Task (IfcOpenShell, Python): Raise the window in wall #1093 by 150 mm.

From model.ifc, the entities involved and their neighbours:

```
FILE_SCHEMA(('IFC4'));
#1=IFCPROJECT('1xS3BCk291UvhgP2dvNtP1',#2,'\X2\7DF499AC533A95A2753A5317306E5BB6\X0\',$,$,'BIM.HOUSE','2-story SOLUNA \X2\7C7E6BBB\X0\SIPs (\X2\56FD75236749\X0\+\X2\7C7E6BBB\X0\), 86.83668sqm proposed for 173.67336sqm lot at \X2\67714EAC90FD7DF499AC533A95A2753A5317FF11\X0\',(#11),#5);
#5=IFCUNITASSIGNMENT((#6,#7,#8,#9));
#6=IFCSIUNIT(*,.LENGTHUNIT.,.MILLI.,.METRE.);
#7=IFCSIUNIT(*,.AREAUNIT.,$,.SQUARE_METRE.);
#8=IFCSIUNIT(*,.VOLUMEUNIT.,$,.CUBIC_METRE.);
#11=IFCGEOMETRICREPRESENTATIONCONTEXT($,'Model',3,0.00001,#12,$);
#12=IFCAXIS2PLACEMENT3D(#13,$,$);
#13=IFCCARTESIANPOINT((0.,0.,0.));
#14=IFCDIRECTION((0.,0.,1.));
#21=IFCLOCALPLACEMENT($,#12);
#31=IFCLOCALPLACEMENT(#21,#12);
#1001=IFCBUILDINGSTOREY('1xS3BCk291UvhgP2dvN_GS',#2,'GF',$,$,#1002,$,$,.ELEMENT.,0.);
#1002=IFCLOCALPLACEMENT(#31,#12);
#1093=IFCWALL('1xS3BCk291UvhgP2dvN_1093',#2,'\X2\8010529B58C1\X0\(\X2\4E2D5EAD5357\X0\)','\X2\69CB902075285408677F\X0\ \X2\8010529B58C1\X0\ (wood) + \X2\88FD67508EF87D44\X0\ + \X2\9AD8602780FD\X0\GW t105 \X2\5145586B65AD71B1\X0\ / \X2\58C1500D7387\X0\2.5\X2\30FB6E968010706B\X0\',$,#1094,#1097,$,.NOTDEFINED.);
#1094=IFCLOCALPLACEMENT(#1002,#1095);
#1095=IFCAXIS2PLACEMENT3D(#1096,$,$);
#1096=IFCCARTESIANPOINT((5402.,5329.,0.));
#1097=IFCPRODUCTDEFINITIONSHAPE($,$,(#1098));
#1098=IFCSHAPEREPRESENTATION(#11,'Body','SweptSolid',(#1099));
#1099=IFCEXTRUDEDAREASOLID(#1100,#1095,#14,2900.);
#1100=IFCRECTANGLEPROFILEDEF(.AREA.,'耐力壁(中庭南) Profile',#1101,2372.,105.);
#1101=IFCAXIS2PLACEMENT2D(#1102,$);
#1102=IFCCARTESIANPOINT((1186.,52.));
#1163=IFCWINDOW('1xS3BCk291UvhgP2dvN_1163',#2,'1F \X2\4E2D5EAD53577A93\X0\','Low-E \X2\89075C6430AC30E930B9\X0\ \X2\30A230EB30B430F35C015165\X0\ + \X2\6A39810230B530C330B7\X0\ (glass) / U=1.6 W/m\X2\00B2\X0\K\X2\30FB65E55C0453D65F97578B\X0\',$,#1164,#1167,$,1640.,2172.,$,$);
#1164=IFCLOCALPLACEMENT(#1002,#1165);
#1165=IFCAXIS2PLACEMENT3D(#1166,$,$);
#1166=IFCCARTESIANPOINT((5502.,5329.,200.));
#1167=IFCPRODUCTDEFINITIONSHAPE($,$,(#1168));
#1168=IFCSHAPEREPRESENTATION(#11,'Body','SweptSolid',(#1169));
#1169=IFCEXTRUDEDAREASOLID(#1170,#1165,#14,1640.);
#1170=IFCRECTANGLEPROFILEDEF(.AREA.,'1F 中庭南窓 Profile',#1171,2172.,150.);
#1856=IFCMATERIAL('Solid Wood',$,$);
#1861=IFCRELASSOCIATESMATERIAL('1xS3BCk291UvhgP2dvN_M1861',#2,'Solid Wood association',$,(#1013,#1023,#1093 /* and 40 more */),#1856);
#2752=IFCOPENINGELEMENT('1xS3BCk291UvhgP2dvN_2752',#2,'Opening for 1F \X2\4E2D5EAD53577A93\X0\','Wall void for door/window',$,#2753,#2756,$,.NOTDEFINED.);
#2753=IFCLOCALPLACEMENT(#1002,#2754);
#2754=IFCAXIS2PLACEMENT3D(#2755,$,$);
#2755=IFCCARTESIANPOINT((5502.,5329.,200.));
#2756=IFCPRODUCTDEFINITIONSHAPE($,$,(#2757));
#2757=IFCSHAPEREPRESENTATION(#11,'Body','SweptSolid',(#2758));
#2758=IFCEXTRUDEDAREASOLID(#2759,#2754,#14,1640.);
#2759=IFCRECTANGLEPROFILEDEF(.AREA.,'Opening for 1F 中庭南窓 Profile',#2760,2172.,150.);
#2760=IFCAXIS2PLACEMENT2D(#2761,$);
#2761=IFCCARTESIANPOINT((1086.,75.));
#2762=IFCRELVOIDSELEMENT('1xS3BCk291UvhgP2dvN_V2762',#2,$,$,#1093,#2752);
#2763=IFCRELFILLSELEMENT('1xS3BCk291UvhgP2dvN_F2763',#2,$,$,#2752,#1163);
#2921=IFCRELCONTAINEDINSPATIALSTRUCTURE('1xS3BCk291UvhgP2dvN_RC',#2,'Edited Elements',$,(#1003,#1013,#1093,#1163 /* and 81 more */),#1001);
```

```python
import numpy as np
import ifcopenshell
import ifcopenshell.api.geometry
import ifcopenshell.util.placement
import ifcopenshell.util.unit

model = ifcopenshell.open("model.ifc")
unit_scale = ifcopenshell.util.unit.calculate_unit_scale(model)

window = model.by_guid("1xS3BCk291UvhgP2dvN_1163")
opening = window.FillsVoids[0].RelatingOpeningElement
dz = 150.0

shift = np.array([0.0, 0.0, dz])
# The window is not placed relative to its opening, so move both.
for product in (opening, window):
    matrix = ifcopenshell.util.placement.get_local_placement(product.ObjectPlacement)
    matrix[:3, 3] += shift
    ifcopenshell.api.geometry.edit_object_placement(model, product=product, matrix=matrix, is_si=False)

print(f"moved by {dz * unit_scale:+.3f} m")

model.write("model_updated.ifc")
```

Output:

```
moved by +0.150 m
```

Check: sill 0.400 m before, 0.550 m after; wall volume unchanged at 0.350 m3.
